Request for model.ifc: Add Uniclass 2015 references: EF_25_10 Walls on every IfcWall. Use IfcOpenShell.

First a look at what the model holds.

```python
import ifcopenshell

model = ifcopenshell.open("model.ifc")
print(model.schema)
print("classifications:", [c.Name for c in model.by_type("IfcClassification")])
for ifc_class in ("IfcDoor", "IfcRoof", "IfcStair", "IfcWall", "IfcWindow"):
    print(ifc_class, len(model.by_type(ifc_class)))
```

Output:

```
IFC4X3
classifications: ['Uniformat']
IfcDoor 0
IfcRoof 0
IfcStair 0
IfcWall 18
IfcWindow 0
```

```python
import ifcopenshell
import ifcopenshell.api.classification

model = ifcopenshell.open("model.ifc")

system = ifcopenshell.api.classification.add_classification(model, classification="Uniclass 2015")

codes = {
    "IfcWall": ("EF_25_10", "Walls"),
}
for ifc_class, (code, name) in codes.items():
    products = model.by_type(ifc_class)
    ifcopenshell.api.classification.add_reference(
        model, products=products, classification=system, identification=code, name=name
    )
    print(code, len(products))

model.write("model_rev.ifc")
```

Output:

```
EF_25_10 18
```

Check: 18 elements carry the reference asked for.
